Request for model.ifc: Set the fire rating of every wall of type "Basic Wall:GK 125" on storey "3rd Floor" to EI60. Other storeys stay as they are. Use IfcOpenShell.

First a look at what the model holds.

```python
import ifcopenshell
import ifcopenshell.util.element

model = ifcopenshell.open("model.ifc")
print(model.schema)
storey = next(s for s in model.by_type("IfcBuildingStorey") if s.Name == "3rd Floor")
walls = [e for e in ifcopenshell.util.element.get_decomposition(storey) if e.is_a("IfcWall")]
seen = {}
for e in walls:
    element_type = ifcopenshell.util.element.get_type(e)
    key = (element_type.Name if element_type != e and element_type else None, ifcopenshell.util.element.get_pset(e, "Pset_WallCommon", "FireRating"))
    seen[key] = seen.get(key, 0) + 1
for (name, value), count in sorted(seen.items(), key=str):
    print(count, "x", name, "|", value)
```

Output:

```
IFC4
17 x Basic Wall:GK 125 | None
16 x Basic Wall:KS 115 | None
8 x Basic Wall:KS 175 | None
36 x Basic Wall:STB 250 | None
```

```python
import ifcopenshell
import ifcopenshell.api.pset
import ifcopenshell.util.element

model = ifcopenshell.open("model.ifc")

storey = next(s for s in model.by_type("IfcBuildingStorey") if s.Name == "3rd Floor")
walls = [e for e in ifcopenshell.util.element.get_decomposition(storey) if e.is_a("IfcWall")]

count = 0
for e in walls:
    element_type = ifcopenshell.util.element.get_type(e)
    if element_type in (None, e) or element_type.Name != "Basic Wall:GK 125":
        continue
    # add_pset returns the element's existing set when there is one.
    pset = ifcopenshell.api.pset.add_pset(model, product=e, name="Pset_WallCommon")
    ifcopenshell.api.pset.edit_pset(model, pset=pset, properties={"FireRating": "EI60"})
    count += 1

print(count, "walls updated")

model.write("model_edited.ifc")
```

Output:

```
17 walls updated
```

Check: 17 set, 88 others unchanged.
